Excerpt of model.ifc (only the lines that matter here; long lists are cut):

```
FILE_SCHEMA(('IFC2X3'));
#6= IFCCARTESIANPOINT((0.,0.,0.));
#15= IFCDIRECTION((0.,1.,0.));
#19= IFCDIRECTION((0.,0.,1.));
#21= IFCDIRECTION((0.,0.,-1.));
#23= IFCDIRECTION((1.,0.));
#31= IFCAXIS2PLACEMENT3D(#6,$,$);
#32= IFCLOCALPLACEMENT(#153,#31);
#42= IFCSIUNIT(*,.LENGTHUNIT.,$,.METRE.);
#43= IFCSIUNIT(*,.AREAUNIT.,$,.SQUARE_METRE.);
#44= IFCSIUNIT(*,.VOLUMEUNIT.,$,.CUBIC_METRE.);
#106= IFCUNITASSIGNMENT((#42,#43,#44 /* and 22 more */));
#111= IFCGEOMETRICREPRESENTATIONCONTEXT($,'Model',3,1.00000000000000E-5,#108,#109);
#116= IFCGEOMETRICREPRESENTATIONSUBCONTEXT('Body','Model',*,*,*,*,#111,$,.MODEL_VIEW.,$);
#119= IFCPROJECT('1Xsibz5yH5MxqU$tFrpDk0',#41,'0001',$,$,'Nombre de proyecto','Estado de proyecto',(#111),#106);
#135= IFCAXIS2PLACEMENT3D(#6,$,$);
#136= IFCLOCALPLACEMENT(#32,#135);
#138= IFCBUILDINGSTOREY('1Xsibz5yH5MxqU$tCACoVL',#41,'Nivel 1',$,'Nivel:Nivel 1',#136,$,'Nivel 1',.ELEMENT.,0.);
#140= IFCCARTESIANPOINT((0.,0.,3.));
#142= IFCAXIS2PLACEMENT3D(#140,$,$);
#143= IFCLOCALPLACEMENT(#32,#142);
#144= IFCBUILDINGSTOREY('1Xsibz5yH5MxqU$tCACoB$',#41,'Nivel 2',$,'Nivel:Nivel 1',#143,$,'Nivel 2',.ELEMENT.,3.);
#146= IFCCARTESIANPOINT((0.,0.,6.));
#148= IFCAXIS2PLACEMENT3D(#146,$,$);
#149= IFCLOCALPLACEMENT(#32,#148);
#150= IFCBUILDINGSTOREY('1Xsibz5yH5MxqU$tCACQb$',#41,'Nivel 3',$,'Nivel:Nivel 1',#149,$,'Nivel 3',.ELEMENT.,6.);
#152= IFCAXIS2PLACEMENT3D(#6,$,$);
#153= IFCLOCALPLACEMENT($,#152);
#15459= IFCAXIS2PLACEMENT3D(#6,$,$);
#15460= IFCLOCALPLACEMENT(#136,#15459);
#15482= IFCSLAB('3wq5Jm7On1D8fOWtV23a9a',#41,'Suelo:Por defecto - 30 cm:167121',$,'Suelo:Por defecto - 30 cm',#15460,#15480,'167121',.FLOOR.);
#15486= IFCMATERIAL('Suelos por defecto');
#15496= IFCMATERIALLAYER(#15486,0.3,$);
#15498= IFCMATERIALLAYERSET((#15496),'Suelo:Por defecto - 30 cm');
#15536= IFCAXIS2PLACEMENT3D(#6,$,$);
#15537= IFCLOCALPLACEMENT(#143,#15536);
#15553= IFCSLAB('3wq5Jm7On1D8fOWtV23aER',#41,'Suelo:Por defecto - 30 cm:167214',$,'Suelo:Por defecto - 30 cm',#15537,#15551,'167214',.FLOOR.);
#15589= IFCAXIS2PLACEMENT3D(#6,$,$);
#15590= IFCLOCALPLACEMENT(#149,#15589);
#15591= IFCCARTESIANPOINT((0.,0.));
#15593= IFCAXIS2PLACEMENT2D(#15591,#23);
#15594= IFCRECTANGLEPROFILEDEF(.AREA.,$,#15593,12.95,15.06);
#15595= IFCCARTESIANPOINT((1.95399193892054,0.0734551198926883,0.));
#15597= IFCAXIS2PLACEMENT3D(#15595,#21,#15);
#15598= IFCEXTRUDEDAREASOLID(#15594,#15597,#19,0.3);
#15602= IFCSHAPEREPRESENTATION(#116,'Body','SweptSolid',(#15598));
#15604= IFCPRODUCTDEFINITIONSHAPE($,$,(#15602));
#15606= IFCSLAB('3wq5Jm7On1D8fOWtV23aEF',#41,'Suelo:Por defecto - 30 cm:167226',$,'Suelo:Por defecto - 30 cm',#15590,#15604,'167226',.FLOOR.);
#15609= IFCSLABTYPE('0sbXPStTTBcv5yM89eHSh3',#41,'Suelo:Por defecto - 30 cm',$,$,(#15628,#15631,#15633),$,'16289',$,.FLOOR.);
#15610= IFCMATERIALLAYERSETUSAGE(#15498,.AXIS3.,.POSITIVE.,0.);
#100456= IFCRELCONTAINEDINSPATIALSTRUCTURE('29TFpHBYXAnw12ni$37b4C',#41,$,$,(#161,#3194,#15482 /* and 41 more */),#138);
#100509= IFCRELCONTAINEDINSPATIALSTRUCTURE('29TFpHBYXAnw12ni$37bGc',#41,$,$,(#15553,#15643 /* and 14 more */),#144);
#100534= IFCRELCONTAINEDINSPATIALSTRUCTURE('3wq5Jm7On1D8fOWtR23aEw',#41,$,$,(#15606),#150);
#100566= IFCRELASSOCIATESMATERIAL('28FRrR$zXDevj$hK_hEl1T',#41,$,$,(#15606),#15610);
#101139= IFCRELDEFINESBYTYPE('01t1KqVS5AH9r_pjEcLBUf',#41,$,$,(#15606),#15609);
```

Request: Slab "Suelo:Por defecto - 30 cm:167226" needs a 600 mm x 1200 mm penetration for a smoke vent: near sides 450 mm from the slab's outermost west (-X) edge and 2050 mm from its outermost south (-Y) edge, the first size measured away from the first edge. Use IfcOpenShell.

```python
import numpy as np
import ifcopenshell
import ifcopenshell.api.feature
import ifcopenshell.api.geometry
import ifcopenshell.api.root
import ifcopenshell.geom
import ifcopenshell.util.placement
import ifcopenshell.util.representation
import ifcopenshell.util.shape
import ifcopenshell.util.unit

model = ifcopenshell.open("model.ifc")
unit_scale = ifcopenshell.util.unit.calculate_unit_scale(model)
settings = ifcopenshell.geom.settings()


def volume(element):
    """Net volume in cubic metres, openings subtracted."""
    shape = ifcopenshell.geom.create_shape(settings, element)
    return ifcopenshell.util.shape.get_volume(shape.geometry)


slab = model.by_guid("3wq5Jm7On1D8fOWtV23aEF")
before = volume(slab)

# Extent in the slab's own axes, in metres. The edges named are its -X and -Y sides.
slab_shape = ifcopenshell.geom.create_shape(settings, slab)
vertices = ifcopenshell.util.shape.get_vertices(slab_shape.geometry)
x_min, y_min, bottom = vertices.min(axis=0)
top = vertices[:, 2].max()

opening = ifcopenshell.api.root.create_entity(model, ifc_class="IfcOpeningElement", name="Smoke vent opening")
context = ifcopenshell.util.representation.get_context(model, "Model", "Body", "MODEL_VIEW")
width, depth = 0.6, 1.2
outline = [(0.0, 0.0), (width, 0.0), (width, depth), (0.0, depth), (0.0, 0.0)]
# Overshoot both faces by 50 mm so the cut is clean.
shape = ifcopenshell.api.geometry.add_slab_representation(
    model, context=context, depth=top - bottom + 0.1, polyline=outline
)
ifcopenshell.api.geometry.assign_representation(model, product=opening, representation=shape)

matrix = ifcopenshell.util.placement.get_local_placement(slab.ObjectPlacement)
matrix[:, 3] = matrix @ np.append(np.array([x_min + 0.45, y_min + 2.05, bottom - 0.05]) / unit_scale, 1.0)
ifcopenshell.api.geometry.edit_object_placement(model, product=opening, matrix=matrix, is_si=False)
ifcopenshell.api.feature.add_feature(model, feature=opening, element=slab)

after = volume(slab)

print(f"slab volume {before:.3f} -> {after:.3f} m3")

model.write("model_edited.ifc")
```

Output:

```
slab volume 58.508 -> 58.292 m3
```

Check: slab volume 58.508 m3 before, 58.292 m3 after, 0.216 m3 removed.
